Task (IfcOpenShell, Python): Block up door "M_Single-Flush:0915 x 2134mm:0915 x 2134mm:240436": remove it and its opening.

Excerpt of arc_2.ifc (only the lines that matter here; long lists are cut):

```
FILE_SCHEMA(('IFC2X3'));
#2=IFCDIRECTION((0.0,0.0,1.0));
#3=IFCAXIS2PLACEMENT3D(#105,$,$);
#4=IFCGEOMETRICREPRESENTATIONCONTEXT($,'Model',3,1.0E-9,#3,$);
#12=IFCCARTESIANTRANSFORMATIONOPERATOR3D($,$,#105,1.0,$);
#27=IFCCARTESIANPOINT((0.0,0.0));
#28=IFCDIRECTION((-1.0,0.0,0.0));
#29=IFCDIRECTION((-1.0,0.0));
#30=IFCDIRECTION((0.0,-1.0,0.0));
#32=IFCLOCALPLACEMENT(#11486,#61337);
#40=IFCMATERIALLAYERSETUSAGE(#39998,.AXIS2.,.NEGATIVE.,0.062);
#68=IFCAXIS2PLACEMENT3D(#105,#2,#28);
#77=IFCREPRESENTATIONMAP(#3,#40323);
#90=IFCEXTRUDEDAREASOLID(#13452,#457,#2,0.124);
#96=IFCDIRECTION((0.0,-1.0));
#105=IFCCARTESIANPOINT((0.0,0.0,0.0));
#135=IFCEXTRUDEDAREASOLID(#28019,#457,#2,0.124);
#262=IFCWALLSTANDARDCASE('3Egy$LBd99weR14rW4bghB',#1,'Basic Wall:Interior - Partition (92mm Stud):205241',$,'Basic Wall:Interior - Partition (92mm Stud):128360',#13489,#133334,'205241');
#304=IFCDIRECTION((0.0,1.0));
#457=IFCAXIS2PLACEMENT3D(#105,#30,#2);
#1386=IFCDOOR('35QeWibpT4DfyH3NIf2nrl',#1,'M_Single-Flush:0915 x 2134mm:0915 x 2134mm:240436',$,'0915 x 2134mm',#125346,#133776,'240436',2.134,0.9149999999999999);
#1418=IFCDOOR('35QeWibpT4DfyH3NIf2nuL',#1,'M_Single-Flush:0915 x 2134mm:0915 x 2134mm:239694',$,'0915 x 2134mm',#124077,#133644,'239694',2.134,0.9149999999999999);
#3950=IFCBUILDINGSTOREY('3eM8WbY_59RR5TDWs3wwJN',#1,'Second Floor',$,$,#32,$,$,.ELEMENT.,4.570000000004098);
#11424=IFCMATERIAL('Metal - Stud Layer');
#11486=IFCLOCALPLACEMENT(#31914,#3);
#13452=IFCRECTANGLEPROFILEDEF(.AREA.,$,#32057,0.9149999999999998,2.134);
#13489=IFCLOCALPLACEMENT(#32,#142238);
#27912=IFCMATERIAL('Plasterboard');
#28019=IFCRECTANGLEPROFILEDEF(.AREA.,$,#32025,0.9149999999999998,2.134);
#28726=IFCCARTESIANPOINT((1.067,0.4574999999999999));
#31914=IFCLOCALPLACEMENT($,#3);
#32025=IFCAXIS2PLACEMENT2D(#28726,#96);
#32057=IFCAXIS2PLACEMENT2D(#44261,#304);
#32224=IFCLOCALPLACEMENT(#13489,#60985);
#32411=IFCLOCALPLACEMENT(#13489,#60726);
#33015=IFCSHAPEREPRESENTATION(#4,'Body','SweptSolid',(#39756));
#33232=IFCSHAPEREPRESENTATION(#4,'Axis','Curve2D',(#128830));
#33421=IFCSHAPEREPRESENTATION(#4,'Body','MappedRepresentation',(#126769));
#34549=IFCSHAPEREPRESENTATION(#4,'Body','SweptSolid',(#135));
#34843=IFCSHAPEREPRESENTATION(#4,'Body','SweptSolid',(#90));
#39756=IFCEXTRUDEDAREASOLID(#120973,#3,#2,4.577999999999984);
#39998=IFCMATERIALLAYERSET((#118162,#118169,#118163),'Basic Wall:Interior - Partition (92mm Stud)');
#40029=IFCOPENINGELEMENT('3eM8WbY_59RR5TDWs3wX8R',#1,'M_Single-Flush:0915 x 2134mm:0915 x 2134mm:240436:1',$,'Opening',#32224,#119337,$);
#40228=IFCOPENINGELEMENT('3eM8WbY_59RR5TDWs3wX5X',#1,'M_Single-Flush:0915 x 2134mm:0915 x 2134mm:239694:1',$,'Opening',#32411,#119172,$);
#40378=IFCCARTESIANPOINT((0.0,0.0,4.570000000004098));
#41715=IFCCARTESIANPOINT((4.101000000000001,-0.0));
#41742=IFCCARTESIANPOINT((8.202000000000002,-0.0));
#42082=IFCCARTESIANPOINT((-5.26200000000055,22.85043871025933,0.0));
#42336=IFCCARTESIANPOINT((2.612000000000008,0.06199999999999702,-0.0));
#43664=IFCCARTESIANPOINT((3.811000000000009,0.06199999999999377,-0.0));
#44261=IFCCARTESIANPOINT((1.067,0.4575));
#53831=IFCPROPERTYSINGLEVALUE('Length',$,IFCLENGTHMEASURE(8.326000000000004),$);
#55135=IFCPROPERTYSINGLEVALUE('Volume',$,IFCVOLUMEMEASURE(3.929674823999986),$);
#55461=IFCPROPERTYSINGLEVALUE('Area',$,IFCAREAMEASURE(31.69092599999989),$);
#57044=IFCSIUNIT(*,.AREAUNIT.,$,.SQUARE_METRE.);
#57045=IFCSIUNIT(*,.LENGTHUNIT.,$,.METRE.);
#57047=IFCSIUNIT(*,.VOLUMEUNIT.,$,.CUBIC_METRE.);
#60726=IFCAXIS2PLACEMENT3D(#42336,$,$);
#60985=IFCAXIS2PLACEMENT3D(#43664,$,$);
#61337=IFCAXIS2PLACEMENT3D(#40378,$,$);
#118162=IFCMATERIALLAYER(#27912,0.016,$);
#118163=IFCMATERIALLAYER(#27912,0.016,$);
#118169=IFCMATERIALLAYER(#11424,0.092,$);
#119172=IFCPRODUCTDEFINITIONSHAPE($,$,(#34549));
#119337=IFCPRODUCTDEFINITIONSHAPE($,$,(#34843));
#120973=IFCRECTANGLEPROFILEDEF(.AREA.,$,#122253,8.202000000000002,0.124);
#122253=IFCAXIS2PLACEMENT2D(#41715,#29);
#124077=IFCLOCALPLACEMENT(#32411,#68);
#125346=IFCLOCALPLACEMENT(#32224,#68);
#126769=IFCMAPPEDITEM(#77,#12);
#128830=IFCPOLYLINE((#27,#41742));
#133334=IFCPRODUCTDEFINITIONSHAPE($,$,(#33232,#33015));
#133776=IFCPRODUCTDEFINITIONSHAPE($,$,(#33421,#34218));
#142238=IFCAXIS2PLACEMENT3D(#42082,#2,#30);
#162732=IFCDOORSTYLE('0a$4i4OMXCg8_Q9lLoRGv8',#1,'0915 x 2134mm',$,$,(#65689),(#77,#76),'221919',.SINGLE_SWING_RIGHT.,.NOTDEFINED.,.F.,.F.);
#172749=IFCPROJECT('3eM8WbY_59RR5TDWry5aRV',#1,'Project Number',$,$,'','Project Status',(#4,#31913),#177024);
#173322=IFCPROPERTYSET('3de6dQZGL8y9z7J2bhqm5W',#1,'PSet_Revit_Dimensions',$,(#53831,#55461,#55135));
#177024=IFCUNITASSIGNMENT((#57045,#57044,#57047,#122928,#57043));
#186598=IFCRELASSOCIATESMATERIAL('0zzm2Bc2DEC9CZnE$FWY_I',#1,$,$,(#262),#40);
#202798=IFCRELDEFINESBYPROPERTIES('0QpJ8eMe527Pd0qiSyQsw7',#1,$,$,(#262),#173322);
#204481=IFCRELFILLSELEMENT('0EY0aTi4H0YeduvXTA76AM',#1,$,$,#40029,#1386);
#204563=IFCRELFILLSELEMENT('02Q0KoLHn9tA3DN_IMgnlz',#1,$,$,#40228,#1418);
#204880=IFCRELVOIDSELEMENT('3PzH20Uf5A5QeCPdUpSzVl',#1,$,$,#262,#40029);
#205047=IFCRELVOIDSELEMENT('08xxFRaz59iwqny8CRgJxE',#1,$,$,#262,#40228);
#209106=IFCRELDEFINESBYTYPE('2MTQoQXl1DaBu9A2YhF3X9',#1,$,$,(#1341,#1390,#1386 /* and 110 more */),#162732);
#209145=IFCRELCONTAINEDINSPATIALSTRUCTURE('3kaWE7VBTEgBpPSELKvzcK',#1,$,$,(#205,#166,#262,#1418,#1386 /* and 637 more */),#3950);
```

```python
import ifcopenshell
import ifcopenshell.api.feature
import ifcopenshell.api.pset
import ifcopenshell.api.root
import ifcopenshell.geom
import ifcopenshell.util.element
import ifcopenshell.util.shape
import ifcopenshell.util.unit

model = ifcopenshell.open("arc_2.ifc")
area_scale = ifcopenshell.util.unit.calculate_unit_scale(model, "AREAUNIT")
volume_scale = ifcopenshell.util.unit.calculate_unit_scale(model, "VOLUMEUNIT")
settings = ifcopenshell.geom.settings()


def volume(element):
    """Net volume in cubic metres, openings subtracted."""
    shape = ifcopenshell.geom.create_shape(settings, element)
    return ifcopenshell.util.shape.get_volume(shape.geometry)


door = model.by_id(1386)
opening = door.FillsVoids[0].RelatingOpeningElement
wall = opening.VoidsElements[0].RelatingBuildingElement
before = volume(wall)

ifcopenshell.api.root.remove_product(model, product=door)
ifcopenshell.api.feature.remove_feature(model, feature=opening)

after = volume(wall)
thickness = 0.124  # wall thickness in metres

# Update the wall's stored quantities.
pset = model.by_id(ifcopenshell.util.element.get_pset(wall, "PSet_Revit_Dimensions", should_inherit=False)["id"])
ifcopenshell.api.pset.edit_pset(model, pset=pset, properties={
    "Area": model.create_entity("IfcAreaMeasure", after / thickness / area_scale),
    "Volume": model.create_entity("IfcVolumeMeasure", after / volume_scale),
})

print(f"wall volume {before:.3f} -> {after:.3f} m3")

model.write("arc_2_edited.ifc")
```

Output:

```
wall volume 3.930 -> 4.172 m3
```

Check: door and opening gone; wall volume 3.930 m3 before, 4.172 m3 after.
